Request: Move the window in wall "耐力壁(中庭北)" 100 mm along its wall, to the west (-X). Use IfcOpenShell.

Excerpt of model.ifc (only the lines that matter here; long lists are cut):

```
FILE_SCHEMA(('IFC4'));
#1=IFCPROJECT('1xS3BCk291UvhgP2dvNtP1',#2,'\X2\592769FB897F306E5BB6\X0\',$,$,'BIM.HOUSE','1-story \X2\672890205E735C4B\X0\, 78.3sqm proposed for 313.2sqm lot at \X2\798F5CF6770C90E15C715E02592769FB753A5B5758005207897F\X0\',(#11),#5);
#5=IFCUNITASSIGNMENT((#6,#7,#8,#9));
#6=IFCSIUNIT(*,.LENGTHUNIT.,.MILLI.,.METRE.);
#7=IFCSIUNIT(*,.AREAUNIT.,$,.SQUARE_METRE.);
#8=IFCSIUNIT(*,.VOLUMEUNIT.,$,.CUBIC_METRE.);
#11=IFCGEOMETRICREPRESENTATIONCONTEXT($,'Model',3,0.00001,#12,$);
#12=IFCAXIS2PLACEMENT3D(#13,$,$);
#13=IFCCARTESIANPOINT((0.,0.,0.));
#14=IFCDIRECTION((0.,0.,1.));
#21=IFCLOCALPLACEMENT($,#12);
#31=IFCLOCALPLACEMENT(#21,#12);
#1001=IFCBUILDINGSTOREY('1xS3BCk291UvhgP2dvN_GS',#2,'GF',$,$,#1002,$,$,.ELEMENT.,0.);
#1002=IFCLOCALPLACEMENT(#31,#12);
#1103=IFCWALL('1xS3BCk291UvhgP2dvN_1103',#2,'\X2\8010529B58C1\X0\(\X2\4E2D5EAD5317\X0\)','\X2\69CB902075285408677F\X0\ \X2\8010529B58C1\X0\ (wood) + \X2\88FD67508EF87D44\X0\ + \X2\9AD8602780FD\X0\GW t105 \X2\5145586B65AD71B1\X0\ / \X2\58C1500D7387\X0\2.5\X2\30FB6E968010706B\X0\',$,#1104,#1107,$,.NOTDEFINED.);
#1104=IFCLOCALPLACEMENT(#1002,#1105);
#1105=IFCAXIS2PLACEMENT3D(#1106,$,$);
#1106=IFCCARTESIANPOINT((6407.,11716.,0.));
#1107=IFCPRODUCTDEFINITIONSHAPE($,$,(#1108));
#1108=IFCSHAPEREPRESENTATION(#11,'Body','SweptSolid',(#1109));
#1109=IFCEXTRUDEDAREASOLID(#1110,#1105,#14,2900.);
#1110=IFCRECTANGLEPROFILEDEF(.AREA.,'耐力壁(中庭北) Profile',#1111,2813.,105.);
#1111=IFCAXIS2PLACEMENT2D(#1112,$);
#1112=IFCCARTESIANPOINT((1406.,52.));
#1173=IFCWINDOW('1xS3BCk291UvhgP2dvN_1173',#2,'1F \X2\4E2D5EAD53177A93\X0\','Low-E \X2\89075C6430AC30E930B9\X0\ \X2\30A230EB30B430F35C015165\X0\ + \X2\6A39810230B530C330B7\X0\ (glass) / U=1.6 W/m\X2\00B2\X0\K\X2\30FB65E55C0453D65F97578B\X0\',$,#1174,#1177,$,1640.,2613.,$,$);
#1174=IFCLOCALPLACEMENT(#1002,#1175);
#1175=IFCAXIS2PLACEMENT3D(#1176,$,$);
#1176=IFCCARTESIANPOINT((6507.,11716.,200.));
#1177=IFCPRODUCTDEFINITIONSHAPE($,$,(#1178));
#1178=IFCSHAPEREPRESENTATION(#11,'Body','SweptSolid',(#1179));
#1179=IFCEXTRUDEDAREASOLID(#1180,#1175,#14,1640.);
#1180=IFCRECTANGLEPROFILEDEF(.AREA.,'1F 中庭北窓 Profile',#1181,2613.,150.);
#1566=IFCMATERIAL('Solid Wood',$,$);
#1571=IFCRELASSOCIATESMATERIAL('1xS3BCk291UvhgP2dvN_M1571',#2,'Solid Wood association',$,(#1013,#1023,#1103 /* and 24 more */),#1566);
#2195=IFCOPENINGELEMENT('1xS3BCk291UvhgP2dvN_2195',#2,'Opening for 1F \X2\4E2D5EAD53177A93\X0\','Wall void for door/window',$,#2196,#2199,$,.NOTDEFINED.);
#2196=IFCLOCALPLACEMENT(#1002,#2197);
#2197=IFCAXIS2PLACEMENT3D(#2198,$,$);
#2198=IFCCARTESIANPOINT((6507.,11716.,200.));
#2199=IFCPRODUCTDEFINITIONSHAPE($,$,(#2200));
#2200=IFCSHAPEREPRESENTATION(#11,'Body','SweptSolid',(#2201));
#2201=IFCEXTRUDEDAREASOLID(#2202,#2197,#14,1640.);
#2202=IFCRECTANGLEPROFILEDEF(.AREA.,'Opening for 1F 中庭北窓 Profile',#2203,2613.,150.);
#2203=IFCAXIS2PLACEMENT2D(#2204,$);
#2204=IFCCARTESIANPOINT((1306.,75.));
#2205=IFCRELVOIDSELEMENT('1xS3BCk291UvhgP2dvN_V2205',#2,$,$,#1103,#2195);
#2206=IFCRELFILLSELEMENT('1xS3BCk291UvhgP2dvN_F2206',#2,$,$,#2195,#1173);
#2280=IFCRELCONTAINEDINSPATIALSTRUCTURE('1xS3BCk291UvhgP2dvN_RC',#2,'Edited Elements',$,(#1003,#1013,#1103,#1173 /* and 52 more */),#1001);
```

```python
import ifcopenshell
import ifcopenshell.api.geometry
import ifcopenshell.util.placement
import ifcopenshell.util.unit

model = ifcopenshell.open("model.ifc")
unit_scale = ifcopenshell.util.unit.calculate_unit_scale(model)

window = model.by_id(1173)
opening = window.FillsVoids[0].RelatingOpeningElement
wall = opening.VoidsElements[0].RelatingBuildingElement

wall_matrix = ifcopenshell.util.placement.get_local_placement(wall.ObjectPlacement)
shift = wall_matrix[:3, 0] * -0.1 / unit_scale
before = ifcopenshell.util.placement.get_local_placement(window.ObjectPlacement)[:3, 3].copy()

# The window is not placed relative to its opening, so move both.
for product in (opening, window):
    matrix = ifcopenshell.util.placement.get_local_placement(product.ObjectPlacement)
    matrix[:3, 3] += shift
    ifcopenshell.api.geometry.edit_object_placement(model, product=product, matrix=matrix, is_si=False)

after = ifcopenshell.util.placement.get_local_placement(window.ObjectPlacement)[:3, 3]
print("window moved by", (after - before).round(3) + 0.0)

model.write("model_updated.ifc")
```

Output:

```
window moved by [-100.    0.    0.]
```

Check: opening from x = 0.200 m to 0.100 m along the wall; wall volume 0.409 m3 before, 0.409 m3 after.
